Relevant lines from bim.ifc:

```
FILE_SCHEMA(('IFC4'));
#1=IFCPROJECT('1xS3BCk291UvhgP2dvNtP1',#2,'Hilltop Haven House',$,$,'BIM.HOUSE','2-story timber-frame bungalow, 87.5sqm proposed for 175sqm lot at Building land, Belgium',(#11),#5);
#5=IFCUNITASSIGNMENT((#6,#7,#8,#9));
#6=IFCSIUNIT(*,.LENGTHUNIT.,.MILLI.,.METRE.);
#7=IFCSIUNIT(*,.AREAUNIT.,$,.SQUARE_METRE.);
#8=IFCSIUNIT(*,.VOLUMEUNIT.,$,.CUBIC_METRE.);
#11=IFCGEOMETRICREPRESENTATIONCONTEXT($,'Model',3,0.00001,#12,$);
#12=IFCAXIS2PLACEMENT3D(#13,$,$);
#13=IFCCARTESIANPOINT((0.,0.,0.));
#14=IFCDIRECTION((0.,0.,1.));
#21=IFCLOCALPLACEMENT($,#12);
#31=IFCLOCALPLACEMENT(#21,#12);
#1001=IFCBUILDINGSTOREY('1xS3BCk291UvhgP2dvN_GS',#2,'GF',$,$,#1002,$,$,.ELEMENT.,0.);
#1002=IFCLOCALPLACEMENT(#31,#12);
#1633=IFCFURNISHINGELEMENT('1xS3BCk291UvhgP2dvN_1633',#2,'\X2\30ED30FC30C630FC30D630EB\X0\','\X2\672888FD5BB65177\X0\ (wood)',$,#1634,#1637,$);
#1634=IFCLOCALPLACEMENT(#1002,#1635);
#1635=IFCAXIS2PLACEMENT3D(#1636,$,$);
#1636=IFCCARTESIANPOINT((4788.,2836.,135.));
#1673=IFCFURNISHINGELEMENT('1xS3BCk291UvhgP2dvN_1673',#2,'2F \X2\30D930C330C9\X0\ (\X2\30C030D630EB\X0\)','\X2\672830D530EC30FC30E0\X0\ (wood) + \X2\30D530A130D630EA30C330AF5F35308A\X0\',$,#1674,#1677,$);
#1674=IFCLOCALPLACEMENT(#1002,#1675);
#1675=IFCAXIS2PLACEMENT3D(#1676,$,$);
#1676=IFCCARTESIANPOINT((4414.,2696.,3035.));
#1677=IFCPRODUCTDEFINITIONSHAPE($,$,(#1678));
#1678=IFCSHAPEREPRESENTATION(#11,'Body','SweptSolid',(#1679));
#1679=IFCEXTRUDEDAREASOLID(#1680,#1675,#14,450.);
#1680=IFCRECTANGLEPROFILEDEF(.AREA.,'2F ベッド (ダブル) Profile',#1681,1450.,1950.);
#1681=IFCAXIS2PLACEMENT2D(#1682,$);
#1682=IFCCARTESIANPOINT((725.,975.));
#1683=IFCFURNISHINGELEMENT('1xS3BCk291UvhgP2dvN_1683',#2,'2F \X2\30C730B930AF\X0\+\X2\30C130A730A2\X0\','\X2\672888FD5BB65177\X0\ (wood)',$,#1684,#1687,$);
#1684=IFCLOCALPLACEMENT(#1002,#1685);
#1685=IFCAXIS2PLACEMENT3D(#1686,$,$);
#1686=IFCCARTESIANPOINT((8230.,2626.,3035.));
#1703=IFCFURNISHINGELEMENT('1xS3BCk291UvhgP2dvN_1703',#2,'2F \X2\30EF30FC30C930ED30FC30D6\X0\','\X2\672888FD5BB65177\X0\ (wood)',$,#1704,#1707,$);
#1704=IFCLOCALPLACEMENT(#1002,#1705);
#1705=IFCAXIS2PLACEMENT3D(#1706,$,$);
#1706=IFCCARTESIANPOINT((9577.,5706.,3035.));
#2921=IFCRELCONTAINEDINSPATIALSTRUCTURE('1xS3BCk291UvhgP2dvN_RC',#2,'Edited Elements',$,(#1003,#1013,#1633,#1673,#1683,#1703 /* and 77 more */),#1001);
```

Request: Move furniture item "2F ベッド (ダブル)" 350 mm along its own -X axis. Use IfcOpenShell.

```python
import ifcopenshell
import ifcopenshell.api.geometry
import ifcopenshell.util.placement
import ifcopenshell.util.unit

model = ifcopenshell.open("bim.ifc")
unit_scale = ifcopenshell.util.unit.calculate_unit_scale(model)

item = model.by_guid("1xS3BCk291UvhgP2dvN_1673")
matrix = ifcopenshell.util.placement.get_local_placement(item.ObjectPlacement)
matrix[:3, 3] -= matrix[:3, 0] * 0.35 / unit_scale
ifcopenshell.api.geometry.edit_object_placement(model, product=item, matrix=matrix, is_si=False)

print(ifcopenshell.util.placement.get_local_placement(item.ObjectPlacement).round(3) + 0.0)

model.write("bim_rev.ifc")
```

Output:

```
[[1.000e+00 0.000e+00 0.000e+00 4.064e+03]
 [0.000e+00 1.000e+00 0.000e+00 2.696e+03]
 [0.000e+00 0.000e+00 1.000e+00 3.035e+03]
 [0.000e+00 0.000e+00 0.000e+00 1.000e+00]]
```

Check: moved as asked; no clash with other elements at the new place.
